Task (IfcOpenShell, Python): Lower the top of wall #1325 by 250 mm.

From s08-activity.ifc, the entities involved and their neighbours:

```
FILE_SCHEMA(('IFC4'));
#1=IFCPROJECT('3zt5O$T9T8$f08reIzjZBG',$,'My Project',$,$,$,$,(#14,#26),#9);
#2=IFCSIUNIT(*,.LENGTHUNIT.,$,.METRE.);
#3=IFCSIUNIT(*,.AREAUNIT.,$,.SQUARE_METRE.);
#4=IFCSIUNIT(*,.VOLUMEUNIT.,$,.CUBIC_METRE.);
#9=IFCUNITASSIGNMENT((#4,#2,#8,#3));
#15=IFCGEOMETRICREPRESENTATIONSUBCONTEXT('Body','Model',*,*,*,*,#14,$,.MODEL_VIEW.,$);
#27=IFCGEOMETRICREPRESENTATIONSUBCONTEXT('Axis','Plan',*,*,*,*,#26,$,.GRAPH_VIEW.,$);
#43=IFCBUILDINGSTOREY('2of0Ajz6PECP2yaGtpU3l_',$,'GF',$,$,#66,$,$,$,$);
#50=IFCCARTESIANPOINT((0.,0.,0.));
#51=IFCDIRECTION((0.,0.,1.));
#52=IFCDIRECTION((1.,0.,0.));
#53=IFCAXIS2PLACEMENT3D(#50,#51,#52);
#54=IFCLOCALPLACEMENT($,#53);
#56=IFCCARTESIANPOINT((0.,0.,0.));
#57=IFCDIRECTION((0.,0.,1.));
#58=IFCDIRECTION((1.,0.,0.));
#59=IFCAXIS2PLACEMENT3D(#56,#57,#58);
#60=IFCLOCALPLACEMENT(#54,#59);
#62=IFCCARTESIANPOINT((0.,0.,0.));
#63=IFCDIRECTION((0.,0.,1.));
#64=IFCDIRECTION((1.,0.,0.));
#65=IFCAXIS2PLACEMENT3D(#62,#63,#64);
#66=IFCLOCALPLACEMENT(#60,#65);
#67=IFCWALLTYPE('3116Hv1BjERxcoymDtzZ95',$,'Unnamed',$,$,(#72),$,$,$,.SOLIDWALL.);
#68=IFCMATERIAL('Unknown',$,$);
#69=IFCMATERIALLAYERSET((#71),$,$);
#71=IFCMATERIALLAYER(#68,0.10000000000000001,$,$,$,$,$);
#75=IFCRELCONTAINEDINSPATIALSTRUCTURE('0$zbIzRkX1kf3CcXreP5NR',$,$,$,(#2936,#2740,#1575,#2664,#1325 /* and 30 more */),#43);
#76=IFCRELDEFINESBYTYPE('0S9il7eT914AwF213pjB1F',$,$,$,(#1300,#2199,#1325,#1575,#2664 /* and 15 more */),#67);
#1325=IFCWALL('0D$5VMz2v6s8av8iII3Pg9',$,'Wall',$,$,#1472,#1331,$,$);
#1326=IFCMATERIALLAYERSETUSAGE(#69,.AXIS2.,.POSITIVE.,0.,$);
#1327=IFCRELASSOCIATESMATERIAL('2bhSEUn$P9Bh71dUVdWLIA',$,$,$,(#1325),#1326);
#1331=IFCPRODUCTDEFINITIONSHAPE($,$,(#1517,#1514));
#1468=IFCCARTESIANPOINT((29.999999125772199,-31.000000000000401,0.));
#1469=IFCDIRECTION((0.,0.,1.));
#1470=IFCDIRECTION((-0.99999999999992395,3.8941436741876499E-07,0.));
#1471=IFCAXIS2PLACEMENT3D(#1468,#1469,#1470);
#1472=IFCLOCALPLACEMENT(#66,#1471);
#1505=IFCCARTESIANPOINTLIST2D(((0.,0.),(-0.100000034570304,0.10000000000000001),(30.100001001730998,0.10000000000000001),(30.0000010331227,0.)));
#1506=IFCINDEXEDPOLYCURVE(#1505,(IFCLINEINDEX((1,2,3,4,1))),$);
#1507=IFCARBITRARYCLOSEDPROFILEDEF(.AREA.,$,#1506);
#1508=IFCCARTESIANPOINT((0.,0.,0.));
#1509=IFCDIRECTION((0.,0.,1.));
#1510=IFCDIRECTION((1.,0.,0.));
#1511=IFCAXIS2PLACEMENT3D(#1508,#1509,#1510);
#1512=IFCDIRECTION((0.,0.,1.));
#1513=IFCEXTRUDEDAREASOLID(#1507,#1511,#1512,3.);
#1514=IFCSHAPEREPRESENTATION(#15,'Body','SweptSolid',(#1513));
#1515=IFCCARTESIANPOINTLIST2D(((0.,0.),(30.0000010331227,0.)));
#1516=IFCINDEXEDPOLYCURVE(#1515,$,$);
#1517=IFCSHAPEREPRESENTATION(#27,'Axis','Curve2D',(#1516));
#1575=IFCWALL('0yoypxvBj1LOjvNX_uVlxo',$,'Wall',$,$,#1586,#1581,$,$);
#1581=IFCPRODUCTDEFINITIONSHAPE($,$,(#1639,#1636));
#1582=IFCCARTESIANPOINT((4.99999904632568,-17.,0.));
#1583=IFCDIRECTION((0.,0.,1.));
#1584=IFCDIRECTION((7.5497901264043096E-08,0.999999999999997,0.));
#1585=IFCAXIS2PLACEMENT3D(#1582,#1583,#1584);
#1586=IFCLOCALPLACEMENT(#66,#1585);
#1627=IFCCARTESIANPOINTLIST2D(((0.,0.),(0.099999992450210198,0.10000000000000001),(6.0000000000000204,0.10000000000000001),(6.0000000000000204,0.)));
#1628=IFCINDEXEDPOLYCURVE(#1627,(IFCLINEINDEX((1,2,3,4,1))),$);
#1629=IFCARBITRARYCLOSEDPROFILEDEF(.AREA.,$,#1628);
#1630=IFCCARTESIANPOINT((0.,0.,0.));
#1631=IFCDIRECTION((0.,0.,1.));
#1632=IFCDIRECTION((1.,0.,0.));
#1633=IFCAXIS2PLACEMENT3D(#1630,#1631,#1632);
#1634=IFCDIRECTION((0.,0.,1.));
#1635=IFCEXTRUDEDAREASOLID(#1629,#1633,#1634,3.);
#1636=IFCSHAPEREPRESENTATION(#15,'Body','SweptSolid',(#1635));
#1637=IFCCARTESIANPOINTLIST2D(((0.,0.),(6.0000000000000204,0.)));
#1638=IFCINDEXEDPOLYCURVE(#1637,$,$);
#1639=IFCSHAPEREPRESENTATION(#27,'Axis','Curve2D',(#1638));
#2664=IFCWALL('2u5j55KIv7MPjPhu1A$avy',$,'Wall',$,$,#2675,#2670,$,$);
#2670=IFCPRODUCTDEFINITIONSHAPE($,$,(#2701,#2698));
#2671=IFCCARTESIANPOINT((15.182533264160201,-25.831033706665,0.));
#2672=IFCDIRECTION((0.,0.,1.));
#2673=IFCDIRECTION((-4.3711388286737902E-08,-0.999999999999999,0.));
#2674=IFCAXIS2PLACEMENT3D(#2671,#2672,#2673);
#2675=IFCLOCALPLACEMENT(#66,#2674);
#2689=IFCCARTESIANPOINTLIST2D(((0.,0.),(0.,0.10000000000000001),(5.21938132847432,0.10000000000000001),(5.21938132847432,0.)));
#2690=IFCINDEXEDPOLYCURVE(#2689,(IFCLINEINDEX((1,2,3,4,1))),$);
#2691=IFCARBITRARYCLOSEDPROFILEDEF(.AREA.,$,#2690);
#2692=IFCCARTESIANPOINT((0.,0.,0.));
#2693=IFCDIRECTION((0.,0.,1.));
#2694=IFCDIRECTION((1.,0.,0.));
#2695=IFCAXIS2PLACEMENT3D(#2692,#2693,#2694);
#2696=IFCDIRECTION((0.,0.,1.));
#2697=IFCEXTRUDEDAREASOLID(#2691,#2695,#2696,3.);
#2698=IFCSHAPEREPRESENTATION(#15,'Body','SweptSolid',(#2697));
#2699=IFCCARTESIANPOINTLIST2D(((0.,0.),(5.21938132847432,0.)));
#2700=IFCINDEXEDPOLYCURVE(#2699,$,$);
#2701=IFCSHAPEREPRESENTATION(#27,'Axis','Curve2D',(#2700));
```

```python
import ifcopenshell
import ifcopenshell.geom
import ifcopenshell.util.representation
import ifcopenshell.util.shape
import ifcopenshell.util.unit

model = ifcopenshell.open("s08-activity.ifc")
unit_scale = ifcopenshell.util.unit.calculate_unit_scale(model)
settings = ifcopenshell.geom.settings()


def volume(element):
    """Net volume in cubic metres, openings subtracted."""
    shape = ifcopenshell.geom.create_shape(settings, element)
    return ifcopenshell.util.shape.get_volume(shape.geometry)


wall = model.by_id(1325)
before = volume(wall)

body = ifcopenshell.util.representation.get_representation(wall, "Model", "Body")
solid = body.Items[0]
old_height = solid.Depth
solid.Depth -= 0.25 / unit_scale
after = volume(wall)

print(f"height {old_height:g} -> {solid.Depth:g}, volume {before:.3f} -> {after:.3f} m3")

model.write("s08-activity_edited.ifc")
```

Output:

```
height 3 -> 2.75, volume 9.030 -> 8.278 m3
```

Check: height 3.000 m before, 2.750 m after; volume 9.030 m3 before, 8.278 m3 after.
